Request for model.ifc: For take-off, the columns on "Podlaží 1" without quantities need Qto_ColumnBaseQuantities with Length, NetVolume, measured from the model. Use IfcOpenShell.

First a look at what the model holds.

```python
import ifcopenshell
import ifcopenshell.util.element
import ifcopenshell.util.unit

model = ifcopenshell.open("model.ifc")
print(model.schema)
for unit_type in ("LENGTHUNIT", "AREAUNIT", "VOLUMEUNIT"):
    print(unit_type, ifcopenshell.util.unit.calculate_unit_scale(model, unit_type))
storey = next(s for s in model.by_type("IfcBuildingStorey") if s.Name == "Podlaží 1")
columns = [e for e in ifcopenshell.util.element.get_decomposition(storey) if e.is_a("IfcColumn")]
for e in sorted(columns, key=lambda e: e.id()):
    print(e.id(), e.is_a(), e.Name, list(ifcopenshell.util.element.get_psets(e, qtos_only=True)), sep=" | ")
```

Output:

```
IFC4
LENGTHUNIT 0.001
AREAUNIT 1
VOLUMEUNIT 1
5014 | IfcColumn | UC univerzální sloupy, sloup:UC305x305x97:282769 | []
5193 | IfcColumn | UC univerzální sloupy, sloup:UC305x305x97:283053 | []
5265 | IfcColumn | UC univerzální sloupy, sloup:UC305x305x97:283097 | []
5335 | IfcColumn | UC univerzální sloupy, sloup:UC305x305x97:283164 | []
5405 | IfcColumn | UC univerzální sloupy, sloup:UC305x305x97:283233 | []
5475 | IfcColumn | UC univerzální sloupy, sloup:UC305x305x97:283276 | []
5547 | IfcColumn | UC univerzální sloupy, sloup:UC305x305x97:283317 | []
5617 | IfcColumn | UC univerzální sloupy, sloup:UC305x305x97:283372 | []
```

```python
import ifcopenshell
import ifcopenshell.api.pset
import ifcopenshell.geom
import ifcopenshell.util.element
import ifcopenshell.util.shape
import ifcopenshell.util.unit

model = ifcopenshell.open("model.ifc")
unit_scale = ifcopenshell.util.unit.calculate_unit_scale(model)
volume_scale = ifcopenshell.util.unit.calculate_unit_scale(model, "VOLUMEUNIT")
settings = ifcopenshell.geom.settings()

storey = next(s for s in model.by_type("IfcBuildingStorey") if s.Name == "Podlaží 1")
columns = [e for e in ifcopenshell.util.element.get_decomposition(storey) if e.is_a("IfcColumn")]

for e in sorted(columns, key=lambda e: e.id()):
    if ifcopenshell.util.element.get_psets(e, qtos_only=True, should_inherit=False):
        continue
    # Geometry comes back in metres, in the element's own axes.
    shape = ifcopenshell.geom.create_shape(settings, e)
    values = {
        "Length": ifcopenshell.util.shape.get_z(shape.geometry) / unit_scale,
        "NetVolume": ifcopenshell.util.shape.get_volume(shape.geometry) / volume_scale,
    }
    qto = ifcopenshell.api.pset.add_qto(model, product=e, name="Qto_ColumnBaseQuantities")
    ifcopenshell.api.pset.edit_qto(model, qto=qto, properties=values)
    print(e.id(), {k: round(v, 3) for k, v in values.items()})

model.write("model_edited.ifc")
```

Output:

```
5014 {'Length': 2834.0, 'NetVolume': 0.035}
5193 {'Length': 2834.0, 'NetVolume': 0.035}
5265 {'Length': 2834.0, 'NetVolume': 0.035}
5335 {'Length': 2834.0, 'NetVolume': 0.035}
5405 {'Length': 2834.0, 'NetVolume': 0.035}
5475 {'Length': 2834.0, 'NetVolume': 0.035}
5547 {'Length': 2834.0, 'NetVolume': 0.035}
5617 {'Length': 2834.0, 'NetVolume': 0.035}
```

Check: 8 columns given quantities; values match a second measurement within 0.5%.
